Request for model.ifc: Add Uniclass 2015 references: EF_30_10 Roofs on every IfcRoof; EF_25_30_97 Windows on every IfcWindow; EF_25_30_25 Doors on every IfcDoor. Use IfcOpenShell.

First a look at what the model holds.

```python
import ifcopenshell

model = ifcopenshell.open("model.ifc")
print(model.schema)
print("classifications:", [c.Name for c in model.by_type("IfcClassification")])
for ifc_class in ("IfcDoor", "IfcRoof", "IfcStair", "IfcWall", "IfcWindow"):
    print(ifc_class, len(model.by_type(ifc_class)))
```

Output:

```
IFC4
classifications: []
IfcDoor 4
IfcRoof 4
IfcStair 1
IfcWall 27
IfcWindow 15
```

```python
import ifcopenshell
import ifcopenshell.api.classification

model = ifcopenshell.open("model.ifc")

system = ifcopenshell.api.classification.add_classification(model, classification="Uniclass 2015")

codes = {
    "IfcRoof": ("EF_30_10", "Roofs"),
    "IfcWindow": ("EF_25_30_97", "Windows"),
    "IfcDoor": ("EF_25_30_25", "Doors"),
}
for ifc_class, (code, name) in codes.items():
    products = model.by_type(ifc_class)
    ifcopenshell.api.classification.add_reference(
        model, products=products, classification=system, identification=code, name=name
    )
    print(code, len(products))

model.write("model-out.ifc")
```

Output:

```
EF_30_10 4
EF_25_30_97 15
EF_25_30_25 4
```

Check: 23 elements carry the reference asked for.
